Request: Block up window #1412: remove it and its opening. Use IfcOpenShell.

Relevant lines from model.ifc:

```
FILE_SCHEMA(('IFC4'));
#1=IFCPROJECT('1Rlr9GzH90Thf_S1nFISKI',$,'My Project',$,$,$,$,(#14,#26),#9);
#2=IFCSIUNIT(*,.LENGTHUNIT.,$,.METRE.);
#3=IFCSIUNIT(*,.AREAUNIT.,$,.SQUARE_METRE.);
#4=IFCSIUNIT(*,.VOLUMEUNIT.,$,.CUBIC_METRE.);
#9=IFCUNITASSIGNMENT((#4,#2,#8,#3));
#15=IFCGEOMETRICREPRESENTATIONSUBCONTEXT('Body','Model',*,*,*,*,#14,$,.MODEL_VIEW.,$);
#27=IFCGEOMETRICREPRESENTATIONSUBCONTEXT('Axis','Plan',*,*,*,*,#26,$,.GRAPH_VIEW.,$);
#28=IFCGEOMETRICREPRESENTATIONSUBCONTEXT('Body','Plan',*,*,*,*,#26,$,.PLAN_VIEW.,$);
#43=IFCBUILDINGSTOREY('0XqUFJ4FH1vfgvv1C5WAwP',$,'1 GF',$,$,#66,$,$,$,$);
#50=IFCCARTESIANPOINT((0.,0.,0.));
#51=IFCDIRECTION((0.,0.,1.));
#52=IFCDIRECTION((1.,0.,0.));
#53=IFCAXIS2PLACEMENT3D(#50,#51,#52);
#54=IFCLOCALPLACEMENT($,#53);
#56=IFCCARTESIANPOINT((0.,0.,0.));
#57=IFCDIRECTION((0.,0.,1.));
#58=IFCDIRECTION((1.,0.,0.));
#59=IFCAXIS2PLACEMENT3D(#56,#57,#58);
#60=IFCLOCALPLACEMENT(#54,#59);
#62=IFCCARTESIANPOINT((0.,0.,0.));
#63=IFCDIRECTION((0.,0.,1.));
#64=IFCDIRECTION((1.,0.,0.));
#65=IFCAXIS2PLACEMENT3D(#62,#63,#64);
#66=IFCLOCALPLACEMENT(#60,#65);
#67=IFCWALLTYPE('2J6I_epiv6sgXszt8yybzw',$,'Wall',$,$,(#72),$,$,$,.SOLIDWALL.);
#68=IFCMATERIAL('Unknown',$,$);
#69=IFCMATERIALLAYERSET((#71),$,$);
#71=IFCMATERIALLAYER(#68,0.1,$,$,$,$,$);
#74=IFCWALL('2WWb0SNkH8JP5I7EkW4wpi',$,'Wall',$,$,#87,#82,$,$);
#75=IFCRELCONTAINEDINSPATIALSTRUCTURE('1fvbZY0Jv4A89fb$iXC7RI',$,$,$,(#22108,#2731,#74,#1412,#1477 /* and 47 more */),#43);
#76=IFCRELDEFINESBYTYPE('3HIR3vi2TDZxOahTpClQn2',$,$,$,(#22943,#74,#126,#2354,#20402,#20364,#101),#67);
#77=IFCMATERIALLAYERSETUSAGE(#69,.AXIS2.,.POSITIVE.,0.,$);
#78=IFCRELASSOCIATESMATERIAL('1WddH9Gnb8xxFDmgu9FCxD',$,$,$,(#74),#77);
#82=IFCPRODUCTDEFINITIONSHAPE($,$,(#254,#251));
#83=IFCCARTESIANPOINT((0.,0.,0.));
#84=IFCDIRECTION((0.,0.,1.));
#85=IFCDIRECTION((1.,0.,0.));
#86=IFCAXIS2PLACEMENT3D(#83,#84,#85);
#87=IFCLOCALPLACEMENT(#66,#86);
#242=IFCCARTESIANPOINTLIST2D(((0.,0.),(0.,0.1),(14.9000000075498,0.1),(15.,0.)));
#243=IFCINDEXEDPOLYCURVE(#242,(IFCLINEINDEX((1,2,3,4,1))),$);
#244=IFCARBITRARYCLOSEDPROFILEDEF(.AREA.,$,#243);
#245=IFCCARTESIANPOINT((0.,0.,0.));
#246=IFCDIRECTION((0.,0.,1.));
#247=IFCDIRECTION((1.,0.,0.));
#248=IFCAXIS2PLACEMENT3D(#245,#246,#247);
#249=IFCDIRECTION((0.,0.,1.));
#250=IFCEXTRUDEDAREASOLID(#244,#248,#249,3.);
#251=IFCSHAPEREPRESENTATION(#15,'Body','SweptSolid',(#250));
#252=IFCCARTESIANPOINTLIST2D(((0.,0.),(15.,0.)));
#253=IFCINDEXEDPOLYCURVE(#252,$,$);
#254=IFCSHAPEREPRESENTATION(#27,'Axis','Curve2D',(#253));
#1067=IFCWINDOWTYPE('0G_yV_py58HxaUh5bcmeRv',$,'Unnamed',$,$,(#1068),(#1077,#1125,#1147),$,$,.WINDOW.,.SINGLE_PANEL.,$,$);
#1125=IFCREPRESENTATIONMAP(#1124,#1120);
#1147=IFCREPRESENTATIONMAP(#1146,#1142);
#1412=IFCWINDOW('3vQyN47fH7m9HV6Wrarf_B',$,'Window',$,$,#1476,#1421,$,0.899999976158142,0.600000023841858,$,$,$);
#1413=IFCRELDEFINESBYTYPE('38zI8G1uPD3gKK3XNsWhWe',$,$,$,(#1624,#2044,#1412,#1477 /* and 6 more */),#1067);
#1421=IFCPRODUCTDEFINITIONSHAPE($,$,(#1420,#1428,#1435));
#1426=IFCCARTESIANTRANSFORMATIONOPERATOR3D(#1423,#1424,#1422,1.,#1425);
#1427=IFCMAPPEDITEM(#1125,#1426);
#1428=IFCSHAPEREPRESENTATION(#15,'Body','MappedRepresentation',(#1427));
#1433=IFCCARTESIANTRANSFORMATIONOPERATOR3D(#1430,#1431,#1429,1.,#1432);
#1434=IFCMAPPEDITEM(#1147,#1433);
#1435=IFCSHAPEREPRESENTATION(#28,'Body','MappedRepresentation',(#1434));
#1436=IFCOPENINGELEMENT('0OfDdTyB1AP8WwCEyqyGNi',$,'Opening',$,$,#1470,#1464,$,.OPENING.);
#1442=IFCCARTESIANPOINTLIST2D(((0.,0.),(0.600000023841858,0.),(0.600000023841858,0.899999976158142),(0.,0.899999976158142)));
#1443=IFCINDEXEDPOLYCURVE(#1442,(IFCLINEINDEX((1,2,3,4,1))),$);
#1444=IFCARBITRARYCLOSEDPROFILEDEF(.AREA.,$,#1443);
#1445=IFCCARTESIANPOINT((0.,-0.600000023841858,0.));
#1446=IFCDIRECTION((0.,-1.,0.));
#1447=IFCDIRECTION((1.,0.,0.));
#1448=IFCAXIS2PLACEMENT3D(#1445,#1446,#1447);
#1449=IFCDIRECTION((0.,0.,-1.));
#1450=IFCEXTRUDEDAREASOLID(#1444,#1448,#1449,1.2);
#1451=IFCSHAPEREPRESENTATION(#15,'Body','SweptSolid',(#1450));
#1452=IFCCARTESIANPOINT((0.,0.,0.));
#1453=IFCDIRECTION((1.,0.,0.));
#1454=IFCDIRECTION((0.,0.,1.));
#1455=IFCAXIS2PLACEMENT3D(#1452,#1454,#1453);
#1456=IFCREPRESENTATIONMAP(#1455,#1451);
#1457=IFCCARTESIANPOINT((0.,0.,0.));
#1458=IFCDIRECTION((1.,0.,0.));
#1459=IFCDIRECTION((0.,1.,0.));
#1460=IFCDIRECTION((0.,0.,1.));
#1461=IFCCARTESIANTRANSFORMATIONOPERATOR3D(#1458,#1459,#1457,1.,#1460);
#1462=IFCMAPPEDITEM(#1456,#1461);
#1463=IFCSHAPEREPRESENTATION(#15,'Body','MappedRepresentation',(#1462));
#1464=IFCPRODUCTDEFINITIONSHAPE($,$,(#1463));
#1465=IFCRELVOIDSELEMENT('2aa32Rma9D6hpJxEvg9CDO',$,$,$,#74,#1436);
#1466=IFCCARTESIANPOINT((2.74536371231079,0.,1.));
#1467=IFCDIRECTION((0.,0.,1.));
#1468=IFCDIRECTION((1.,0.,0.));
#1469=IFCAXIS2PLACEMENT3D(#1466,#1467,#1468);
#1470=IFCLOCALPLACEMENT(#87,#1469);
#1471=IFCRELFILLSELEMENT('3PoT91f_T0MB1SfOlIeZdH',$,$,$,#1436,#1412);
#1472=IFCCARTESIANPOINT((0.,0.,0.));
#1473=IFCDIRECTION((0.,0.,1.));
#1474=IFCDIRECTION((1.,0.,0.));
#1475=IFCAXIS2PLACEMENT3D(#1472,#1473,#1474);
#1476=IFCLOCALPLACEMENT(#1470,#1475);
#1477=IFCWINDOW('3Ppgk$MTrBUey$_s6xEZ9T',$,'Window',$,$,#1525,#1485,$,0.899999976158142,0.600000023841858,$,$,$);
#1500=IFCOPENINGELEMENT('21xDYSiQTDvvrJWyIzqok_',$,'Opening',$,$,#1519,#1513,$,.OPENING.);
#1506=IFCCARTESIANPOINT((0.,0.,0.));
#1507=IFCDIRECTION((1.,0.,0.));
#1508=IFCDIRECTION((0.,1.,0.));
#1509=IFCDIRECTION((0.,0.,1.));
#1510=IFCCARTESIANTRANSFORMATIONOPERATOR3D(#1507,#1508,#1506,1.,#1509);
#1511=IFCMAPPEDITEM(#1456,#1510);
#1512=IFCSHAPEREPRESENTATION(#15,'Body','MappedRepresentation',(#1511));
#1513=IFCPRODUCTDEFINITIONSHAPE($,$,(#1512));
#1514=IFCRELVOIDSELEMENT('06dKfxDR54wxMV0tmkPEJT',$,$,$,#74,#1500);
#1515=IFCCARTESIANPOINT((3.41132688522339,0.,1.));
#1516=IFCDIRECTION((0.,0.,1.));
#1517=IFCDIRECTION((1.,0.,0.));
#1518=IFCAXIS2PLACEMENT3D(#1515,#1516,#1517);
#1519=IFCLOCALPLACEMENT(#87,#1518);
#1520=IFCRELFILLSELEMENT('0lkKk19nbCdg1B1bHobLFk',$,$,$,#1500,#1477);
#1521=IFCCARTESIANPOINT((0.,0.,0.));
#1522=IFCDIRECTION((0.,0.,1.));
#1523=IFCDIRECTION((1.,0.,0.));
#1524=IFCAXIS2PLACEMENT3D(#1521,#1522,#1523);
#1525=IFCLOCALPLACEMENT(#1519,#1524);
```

```python
import ifcopenshell
import ifcopenshell.api.feature
import ifcopenshell.api.root
import ifcopenshell.geom
import ifcopenshell.util.shape

model = ifcopenshell.open("model.ifc")
settings = ifcopenshell.geom.settings()


def volume(element):
    """Net volume in cubic metres, openings subtracted."""
    shape = ifcopenshell.geom.create_shape(settings, element)
    return ifcopenshell.util.shape.get_volume(shape.geometry)


window = model.by_guid("3vQyN47fH7m9HV6Wrarf_B")
opening = window.FillsVoids[0].RelatingOpeningElement
wall = opening.VoidsElements[0].RelatingBuildingElement
before = volume(wall)

ifcopenshell.api.root.remove_product(model, product=window)
ifcopenshell.api.feature.remove_feature(model, feature=opening)

after = volume(wall)

print(f"wall volume {before:.3f} -> {after:.3f} m3")

model.write("model_updated.ifc")
```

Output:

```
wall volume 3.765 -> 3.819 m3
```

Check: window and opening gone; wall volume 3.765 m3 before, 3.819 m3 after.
